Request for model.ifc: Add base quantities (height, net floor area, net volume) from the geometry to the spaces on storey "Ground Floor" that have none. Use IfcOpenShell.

First a look at what the model holds.

```python
import ifcopenshell
import ifcopenshell.util.element
import ifcopenshell.util.unit

model = ifcopenshell.open("model.ifc")
print(model.schema)
for unit_type in ("LENGTHUNIT", "AREAUNIT", "VOLUMEUNIT"):
    print(unit_type, ifcopenshell.util.unit.calculate_unit_scale(model, unit_type))
storey = next(s for s in model.by_type("IfcBuildingStorey") if s.Name == "Ground Floor")
spaces = [e for e in ifcopenshell.util.element.get_decomposition(storey) if e.is_a("IfcSpace")]
for e in sorted(spaces, key=lambda e: e.id()):
    print(e.id(), e.is_a(), e.Name, list(ifcopenshell.util.element.get_psets(e, qtos_only=True)), sep=" | ")
```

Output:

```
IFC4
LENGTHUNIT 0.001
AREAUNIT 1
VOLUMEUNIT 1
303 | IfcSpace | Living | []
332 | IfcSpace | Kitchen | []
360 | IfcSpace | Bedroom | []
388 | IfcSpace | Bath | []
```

```python
import ifcopenshell
import ifcopenshell.api.pset
import ifcopenshell.geom
import ifcopenshell.util.element
import ifcopenshell.util.shape
import ifcopenshell.util.unit

model = ifcopenshell.open("model.ifc")
unit_scale = ifcopenshell.util.unit.calculate_unit_scale(model)
area_scale = ifcopenshell.util.unit.calculate_unit_scale(model, "AREAUNIT")
volume_scale = ifcopenshell.util.unit.calculate_unit_scale(model, "VOLUMEUNIT")
settings = ifcopenshell.geom.settings()

storey = next(s for s in model.by_type("IfcBuildingStorey") if s.Name == "Ground Floor")
spaces = [e for e in ifcopenshell.util.element.get_decomposition(storey) if e.is_a("IfcSpace")]

for e in sorted(spaces, key=lambda e: e.id()):
    if ifcopenshell.util.element.get_psets(e, qtos_only=True, should_inherit=False):
        continue
    # Geometry comes back in metres, in the element's own axes.
    shape = ifcopenshell.geom.create_shape(settings, e)
    values = {
        "Height": ifcopenshell.util.shape.get_z(shape.geometry) / unit_scale,
        "NetFloorArea": ifcopenshell.util.shape.get_footprint_area(shape.geometry) / area_scale,
        "NetVolume": ifcopenshell.util.shape.get_volume(shape.geometry) / volume_scale,
    }
    qto = ifcopenshell.api.pset.add_qto(model, product=e, name="Qto_SpaceBaseQuantities")
    ifcopenshell.api.pset.edit_qto(model, qto=qto, properties=values)
    print(e.id(), {k: round(v, 3) for k, v in values.items()})

model.write("model-out.ifc")
```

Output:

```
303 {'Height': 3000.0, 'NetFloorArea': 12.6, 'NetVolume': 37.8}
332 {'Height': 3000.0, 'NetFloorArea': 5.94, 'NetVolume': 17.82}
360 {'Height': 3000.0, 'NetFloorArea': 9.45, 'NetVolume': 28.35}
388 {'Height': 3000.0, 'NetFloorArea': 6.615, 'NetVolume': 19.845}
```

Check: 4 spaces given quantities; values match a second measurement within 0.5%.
